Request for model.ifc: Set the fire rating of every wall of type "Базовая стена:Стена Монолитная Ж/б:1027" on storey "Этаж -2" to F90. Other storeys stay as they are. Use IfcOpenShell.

First a look at what the model holds.

```python
import ifcopenshell
import ifcopenshell.util.element

model = ifcopenshell.open("model.ifc")
print(model.schema)
storey = next(s for s in model.by_type("IfcBuildingStorey") if s.Name == "Этаж -2")
walls = [e for e in ifcopenshell.util.element.get_decomposition(storey) if e.is_a("IfcWall")]
seen = {}
for e in walls:
    element_type = ifcopenshell.util.element.get_type(e)
    key = (element_type.Name if element_type != e and element_type else None, ifcopenshell.util.element.get_pset(e, "Pset_WallCommon", "FireRating"))
    seen[key] = seen.get(key, 0) + 1
for (name, value), count in sorted(seen.items(), key=str):
    print(count, "x", name, "|", value)
```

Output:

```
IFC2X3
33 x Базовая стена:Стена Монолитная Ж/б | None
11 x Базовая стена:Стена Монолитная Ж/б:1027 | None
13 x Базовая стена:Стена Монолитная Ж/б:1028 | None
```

```python
import ifcopenshell
import ifcopenshell.api.pset
import ifcopenshell.util.element

model = ifcopenshell.open("model.ifc")

storey = next(s for s in model.by_type("IfcBuildingStorey") if s.Name == "Этаж -2")
walls = [e for e in ifcopenshell.util.element.get_decomposition(storey) if e.is_a("IfcWall")]

count = 0
for e in walls:
    element_type = ifcopenshell.util.element.get_type(e)
    if element_type in (None, e) or element_type.Name != "Базовая стена:Стена Монолитная Ж/б:1027":
        continue
    # add_pset returns the element's existing set when there is one.
    pset = ifcopenshell.api.pset.add_pset(model, product=e, name="Pset_WallCommon")
    ifcopenshell.api.pset.edit_pset(model, pset=pset, properties={"FireRating": "F90"})
    count += 1

print(count, "walls updated")

model.write("model_v2.ifc")
```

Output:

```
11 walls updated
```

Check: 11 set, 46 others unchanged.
